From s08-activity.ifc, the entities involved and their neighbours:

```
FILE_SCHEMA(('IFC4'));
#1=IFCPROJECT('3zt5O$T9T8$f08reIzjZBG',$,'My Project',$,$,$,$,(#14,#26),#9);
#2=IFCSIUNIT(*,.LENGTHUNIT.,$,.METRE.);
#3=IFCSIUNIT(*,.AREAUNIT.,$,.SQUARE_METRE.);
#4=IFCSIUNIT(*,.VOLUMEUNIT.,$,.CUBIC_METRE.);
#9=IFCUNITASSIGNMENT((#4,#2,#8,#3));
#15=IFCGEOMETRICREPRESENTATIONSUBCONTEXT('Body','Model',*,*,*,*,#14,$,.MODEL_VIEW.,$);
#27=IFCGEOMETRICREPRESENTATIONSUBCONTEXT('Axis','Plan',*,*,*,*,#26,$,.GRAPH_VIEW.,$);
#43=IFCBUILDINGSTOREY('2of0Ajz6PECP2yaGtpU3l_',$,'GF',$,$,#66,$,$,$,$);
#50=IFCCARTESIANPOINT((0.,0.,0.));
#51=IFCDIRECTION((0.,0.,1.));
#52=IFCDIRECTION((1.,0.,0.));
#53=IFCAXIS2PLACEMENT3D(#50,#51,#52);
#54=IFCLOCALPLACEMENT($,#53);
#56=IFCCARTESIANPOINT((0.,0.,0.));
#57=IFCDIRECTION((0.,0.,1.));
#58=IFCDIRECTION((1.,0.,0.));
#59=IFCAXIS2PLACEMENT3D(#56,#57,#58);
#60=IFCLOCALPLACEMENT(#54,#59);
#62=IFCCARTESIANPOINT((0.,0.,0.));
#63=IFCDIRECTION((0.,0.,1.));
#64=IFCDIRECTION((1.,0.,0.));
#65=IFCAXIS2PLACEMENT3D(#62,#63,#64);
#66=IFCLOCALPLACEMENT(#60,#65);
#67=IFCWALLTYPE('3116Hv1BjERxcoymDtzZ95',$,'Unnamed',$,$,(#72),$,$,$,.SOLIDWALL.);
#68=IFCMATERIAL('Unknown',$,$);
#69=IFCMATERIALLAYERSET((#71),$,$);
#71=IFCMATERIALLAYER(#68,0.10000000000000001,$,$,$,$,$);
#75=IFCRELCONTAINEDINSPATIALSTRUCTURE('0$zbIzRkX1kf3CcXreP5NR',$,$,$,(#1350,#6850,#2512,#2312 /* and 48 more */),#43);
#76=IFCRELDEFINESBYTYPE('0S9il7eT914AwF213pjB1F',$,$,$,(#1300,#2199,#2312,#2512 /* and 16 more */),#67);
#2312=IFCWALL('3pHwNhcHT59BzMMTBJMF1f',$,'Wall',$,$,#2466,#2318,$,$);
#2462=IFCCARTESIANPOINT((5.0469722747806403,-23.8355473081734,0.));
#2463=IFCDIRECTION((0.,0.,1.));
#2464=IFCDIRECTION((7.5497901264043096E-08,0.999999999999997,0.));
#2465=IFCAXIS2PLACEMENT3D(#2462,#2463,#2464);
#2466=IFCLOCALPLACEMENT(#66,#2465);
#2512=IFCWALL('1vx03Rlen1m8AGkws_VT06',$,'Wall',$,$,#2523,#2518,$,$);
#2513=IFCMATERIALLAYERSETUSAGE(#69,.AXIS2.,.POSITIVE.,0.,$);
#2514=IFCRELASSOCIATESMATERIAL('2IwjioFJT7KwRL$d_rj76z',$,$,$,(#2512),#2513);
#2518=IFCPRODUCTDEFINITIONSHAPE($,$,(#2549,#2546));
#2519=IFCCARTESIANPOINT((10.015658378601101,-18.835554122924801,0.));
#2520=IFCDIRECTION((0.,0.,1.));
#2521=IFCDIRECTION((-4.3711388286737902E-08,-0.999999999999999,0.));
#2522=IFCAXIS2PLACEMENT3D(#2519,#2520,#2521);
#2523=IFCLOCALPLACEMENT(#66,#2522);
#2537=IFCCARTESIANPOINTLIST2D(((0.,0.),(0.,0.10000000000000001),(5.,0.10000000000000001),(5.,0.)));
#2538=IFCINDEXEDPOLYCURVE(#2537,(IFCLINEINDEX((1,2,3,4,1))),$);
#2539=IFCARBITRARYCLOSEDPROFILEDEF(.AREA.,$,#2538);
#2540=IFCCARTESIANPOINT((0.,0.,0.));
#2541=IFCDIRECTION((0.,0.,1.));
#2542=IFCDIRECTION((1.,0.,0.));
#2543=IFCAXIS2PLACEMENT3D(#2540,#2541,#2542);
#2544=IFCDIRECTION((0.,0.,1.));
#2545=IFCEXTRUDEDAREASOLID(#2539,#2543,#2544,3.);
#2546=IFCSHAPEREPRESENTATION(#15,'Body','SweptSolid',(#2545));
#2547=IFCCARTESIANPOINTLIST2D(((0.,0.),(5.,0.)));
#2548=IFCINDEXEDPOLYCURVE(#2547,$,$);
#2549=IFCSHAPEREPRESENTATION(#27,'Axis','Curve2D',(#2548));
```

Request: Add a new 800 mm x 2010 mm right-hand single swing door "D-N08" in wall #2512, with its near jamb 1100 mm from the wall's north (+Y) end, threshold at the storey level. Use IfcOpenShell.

```python
import numpy as np
import ifcopenshell
import ifcopenshell.api.feature
import ifcopenshell.api.geometry
import ifcopenshell.api.root
import ifcopenshell.api.spatial
import ifcopenshell.geom
import ifcopenshell.util.element
import ifcopenshell.util.placement
import ifcopenshell.util.representation
import ifcopenshell.util.shape
import ifcopenshell.util.unit

model = ifcopenshell.open("s08-activity.ifc")
unit_scale = ifcopenshell.util.unit.calculate_unit_scale(model)
settings = ifcopenshell.geom.settings()


def volume(element):
    """Net volume in cubic metres, openings subtracted."""
    shape = ifcopenshell.geom.create_shape(settings, element)
    return ifcopenshell.util.shape.get_volume(shape.geometry)


wall = model.by_guid("1vx03Rlen1m8AGkws_VT06")
storey = ifcopenshell.util.element.get_container(wall, ifc_class="IfcBuildingStorey")
context = ifcopenshell.util.representation.get_context(model, "Model", "Body", "MODEL_VIEW")
before = volume(wall)

width, height, from_end, sill = 0.8, 2.01, 1.1, 0.0  # metres

# The wall runs along its own X axis, and the end named is its -X end.
wall_shape = ifcopenshell.geom.create_shape(settings, wall)
x, y, z = ifcopenshell.util.shape.get_vertices(wall_shape.geometry).T
start = x.min() + from_end
face, thickness = float(y.min()), float(y.max() - y.min())
wall_matrix = ifcopenshell.util.placement.get_local_placement(wall.ObjectPlacement)
level = ifcopenshell.util.placement.get_local_placement(storey.ObjectPlacement)[2, 3]


def in_wall(x, y):
    """Placement at x, y metres in the wall's axes, at sill height."""
    matrix = wall_matrix.copy()
    matrix[:, 3] = wall_matrix @ np.array([x / unit_scale, y / unit_scale, 0.0, 1.0])
    matrix[2, 3] = level + sill / unit_scale
    return matrix


# Opening: a box that overshoots both wall faces by 50 mm.
opening = ifcopenshell.api.root.create_entity(model, ifc_class="IfcOpeningElement", predefined_type="OPENING")
box = ifcopenshell.api.geometry.add_wall_representation(
    model, context=context, length=width, height=height, thickness=thickness + 0.1
)
ifcopenshell.api.geometry.assign_representation(model, product=opening, representation=box)
ifcopenshell.api.geometry.edit_object_placement(model, product=opening, matrix=in_wall(start, face - 0.05), is_si=False)
ifcopenshell.api.feature.add_feature(model, feature=opening, element=wall)

door = ifcopenshell.api.root.create_entity(model, ifc_class="IfcDoor", name="D-N08", predefined_type="DOOR")
door.OverallWidth, door.OverallHeight = width / unit_scale, height / unit_scale
door.OperationType = "SINGLE_SWING_RIGHT"
body = ifcopenshell.api.geometry.add_door_representation(
    model,
    context=context,
    overall_width=door.OverallWidth,
    overall_height=door.OverallHeight,
    operation_type="SINGLE_SWING_RIGHT",
    lining_properties={"LiningDepth": thickness / unit_scale, "ThresholdDepth": thickness / unit_scale},
)
ifcopenshell.api.geometry.assign_representation(model, product=door, representation=body)
ifcopenshell.api.spatial.assign_container(model, products=[door], relating_structure=storey)
ifcopenshell.api.feature.add_filling(model, opening=opening, element=door)

# The lining spans the wall, so the door starts at the wall face.
ifcopenshell.api.geometry.edit_object_placement(model, product=door, matrix=in_wall(start, face), is_si=False)

after = volume(wall)

print(f"wall volume {before:.3f} -> {after:.3f} m3")

model.write("s08-activity_v2.ifc")
```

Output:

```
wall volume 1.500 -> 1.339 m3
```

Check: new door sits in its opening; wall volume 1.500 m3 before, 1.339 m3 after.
